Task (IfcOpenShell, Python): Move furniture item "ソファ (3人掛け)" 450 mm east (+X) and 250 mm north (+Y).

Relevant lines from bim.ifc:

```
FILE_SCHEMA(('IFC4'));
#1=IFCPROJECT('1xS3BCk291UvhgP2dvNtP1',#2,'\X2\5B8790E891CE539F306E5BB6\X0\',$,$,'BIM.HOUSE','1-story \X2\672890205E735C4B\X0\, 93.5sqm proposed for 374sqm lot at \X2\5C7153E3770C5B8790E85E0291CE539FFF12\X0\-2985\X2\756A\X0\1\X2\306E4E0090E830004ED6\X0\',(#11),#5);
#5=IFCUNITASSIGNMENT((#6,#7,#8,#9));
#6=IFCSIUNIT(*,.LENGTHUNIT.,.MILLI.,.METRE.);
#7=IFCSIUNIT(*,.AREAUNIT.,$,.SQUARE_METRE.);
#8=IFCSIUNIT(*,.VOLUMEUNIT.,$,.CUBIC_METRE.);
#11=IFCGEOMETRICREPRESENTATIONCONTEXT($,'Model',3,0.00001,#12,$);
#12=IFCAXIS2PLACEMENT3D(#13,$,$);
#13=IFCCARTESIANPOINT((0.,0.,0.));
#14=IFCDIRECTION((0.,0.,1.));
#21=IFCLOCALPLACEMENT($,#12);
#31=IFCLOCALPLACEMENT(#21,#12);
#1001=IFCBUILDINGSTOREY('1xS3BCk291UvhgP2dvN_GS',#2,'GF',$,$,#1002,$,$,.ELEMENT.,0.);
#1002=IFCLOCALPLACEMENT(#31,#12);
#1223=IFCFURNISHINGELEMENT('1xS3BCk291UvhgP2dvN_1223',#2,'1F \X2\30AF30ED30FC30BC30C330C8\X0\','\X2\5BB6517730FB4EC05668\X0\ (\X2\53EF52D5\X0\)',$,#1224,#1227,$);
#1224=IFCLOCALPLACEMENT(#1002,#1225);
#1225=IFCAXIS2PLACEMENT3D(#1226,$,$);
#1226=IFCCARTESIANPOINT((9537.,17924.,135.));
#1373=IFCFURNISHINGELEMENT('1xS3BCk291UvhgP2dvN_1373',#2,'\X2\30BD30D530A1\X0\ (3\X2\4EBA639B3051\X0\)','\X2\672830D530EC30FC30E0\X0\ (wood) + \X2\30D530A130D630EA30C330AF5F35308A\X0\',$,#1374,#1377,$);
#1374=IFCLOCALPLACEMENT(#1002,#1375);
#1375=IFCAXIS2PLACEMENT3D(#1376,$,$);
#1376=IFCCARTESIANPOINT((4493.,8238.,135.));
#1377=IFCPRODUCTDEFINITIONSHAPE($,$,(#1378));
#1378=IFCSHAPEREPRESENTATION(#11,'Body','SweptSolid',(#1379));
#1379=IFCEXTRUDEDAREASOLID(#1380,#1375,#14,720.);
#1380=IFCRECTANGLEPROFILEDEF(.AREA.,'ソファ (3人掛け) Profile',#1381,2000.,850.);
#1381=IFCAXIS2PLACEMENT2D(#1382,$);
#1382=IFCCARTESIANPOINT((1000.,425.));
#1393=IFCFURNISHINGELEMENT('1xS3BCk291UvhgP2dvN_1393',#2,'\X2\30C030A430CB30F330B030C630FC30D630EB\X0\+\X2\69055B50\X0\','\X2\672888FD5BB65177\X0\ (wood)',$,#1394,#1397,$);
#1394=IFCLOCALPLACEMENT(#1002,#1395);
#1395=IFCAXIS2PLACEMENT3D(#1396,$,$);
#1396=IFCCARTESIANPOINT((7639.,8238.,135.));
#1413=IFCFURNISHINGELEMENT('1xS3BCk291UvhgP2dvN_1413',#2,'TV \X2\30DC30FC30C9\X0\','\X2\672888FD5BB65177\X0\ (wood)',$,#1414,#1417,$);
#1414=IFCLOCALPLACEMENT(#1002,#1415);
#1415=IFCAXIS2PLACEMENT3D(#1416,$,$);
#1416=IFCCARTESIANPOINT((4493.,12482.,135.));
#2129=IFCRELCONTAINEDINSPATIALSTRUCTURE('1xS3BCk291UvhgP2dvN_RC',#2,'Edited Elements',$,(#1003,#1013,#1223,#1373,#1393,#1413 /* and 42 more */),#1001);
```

```python
import ifcopenshell
import ifcopenshell.api.geometry
import ifcopenshell.util.placement

model = ifcopenshell.open("bim.ifc")

item = model.by_id(1373)
matrix = ifcopenshell.util.placement.get_local_placement(item.ObjectPlacement)
matrix[0, 3] += 450.0
matrix[1, 3] += 250.0
ifcopenshell.api.geometry.edit_object_placement(model, product=item, matrix=matrix, is_si=False)

print(ifcopenshell.util.placement.get_local_placement(item.ObjectPlacement).round(3) + 0.0)

model.write("bim_updated.ifc")
```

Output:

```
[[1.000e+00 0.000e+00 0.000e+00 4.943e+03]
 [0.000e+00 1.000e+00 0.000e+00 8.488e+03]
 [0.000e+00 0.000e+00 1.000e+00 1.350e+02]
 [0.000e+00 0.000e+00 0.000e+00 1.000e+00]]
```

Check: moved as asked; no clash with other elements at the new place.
